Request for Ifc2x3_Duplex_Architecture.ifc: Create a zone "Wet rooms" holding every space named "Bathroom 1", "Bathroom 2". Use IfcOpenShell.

First a look at what the model holds.

```python
import ifcopenshell

model = ifcopenshell.open("Ifc2x3_Duplex_Architecture.ifc")
print(model.schema)
seen = {}
for space in model.by_type("IfcSpace"):
    seen[space.LongName] = seen.get(space.LongName, 0) + 1
for name, count in sorted(seen.items(), key=str):
    print(count, "x", name)
print("zones:", [z.Name for z in model.by_type("IfcZone")][:20])
```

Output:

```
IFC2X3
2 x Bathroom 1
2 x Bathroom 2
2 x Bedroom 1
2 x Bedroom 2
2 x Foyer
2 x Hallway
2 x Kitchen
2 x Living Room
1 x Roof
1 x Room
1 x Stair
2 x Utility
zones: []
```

```python
import ifcopenshell
import ifcopenshell.api.group
import ifcopenshell.api.root

model = ifcopenshell.open("Ifc2x3_Duplex_Architecture.ifc")

names = {"Bathroom 1", "Bathroom 2"}
spaces = [s for s in model.by_type("IfcSpace") if s.LongName in names]

zone = ifcopenshell.api.root.create_entity(model, ifc_class="IfcZone", name="Wet rooms")
ifcopenshell.api.group.assign_group(model, products=spaces, group=zone)
print(len(spaces), "spaces in", zone.Name)

model.write("Ifc2x3_Duplex_Architecture_updated.ifc")
```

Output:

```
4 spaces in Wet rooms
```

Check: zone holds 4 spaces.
